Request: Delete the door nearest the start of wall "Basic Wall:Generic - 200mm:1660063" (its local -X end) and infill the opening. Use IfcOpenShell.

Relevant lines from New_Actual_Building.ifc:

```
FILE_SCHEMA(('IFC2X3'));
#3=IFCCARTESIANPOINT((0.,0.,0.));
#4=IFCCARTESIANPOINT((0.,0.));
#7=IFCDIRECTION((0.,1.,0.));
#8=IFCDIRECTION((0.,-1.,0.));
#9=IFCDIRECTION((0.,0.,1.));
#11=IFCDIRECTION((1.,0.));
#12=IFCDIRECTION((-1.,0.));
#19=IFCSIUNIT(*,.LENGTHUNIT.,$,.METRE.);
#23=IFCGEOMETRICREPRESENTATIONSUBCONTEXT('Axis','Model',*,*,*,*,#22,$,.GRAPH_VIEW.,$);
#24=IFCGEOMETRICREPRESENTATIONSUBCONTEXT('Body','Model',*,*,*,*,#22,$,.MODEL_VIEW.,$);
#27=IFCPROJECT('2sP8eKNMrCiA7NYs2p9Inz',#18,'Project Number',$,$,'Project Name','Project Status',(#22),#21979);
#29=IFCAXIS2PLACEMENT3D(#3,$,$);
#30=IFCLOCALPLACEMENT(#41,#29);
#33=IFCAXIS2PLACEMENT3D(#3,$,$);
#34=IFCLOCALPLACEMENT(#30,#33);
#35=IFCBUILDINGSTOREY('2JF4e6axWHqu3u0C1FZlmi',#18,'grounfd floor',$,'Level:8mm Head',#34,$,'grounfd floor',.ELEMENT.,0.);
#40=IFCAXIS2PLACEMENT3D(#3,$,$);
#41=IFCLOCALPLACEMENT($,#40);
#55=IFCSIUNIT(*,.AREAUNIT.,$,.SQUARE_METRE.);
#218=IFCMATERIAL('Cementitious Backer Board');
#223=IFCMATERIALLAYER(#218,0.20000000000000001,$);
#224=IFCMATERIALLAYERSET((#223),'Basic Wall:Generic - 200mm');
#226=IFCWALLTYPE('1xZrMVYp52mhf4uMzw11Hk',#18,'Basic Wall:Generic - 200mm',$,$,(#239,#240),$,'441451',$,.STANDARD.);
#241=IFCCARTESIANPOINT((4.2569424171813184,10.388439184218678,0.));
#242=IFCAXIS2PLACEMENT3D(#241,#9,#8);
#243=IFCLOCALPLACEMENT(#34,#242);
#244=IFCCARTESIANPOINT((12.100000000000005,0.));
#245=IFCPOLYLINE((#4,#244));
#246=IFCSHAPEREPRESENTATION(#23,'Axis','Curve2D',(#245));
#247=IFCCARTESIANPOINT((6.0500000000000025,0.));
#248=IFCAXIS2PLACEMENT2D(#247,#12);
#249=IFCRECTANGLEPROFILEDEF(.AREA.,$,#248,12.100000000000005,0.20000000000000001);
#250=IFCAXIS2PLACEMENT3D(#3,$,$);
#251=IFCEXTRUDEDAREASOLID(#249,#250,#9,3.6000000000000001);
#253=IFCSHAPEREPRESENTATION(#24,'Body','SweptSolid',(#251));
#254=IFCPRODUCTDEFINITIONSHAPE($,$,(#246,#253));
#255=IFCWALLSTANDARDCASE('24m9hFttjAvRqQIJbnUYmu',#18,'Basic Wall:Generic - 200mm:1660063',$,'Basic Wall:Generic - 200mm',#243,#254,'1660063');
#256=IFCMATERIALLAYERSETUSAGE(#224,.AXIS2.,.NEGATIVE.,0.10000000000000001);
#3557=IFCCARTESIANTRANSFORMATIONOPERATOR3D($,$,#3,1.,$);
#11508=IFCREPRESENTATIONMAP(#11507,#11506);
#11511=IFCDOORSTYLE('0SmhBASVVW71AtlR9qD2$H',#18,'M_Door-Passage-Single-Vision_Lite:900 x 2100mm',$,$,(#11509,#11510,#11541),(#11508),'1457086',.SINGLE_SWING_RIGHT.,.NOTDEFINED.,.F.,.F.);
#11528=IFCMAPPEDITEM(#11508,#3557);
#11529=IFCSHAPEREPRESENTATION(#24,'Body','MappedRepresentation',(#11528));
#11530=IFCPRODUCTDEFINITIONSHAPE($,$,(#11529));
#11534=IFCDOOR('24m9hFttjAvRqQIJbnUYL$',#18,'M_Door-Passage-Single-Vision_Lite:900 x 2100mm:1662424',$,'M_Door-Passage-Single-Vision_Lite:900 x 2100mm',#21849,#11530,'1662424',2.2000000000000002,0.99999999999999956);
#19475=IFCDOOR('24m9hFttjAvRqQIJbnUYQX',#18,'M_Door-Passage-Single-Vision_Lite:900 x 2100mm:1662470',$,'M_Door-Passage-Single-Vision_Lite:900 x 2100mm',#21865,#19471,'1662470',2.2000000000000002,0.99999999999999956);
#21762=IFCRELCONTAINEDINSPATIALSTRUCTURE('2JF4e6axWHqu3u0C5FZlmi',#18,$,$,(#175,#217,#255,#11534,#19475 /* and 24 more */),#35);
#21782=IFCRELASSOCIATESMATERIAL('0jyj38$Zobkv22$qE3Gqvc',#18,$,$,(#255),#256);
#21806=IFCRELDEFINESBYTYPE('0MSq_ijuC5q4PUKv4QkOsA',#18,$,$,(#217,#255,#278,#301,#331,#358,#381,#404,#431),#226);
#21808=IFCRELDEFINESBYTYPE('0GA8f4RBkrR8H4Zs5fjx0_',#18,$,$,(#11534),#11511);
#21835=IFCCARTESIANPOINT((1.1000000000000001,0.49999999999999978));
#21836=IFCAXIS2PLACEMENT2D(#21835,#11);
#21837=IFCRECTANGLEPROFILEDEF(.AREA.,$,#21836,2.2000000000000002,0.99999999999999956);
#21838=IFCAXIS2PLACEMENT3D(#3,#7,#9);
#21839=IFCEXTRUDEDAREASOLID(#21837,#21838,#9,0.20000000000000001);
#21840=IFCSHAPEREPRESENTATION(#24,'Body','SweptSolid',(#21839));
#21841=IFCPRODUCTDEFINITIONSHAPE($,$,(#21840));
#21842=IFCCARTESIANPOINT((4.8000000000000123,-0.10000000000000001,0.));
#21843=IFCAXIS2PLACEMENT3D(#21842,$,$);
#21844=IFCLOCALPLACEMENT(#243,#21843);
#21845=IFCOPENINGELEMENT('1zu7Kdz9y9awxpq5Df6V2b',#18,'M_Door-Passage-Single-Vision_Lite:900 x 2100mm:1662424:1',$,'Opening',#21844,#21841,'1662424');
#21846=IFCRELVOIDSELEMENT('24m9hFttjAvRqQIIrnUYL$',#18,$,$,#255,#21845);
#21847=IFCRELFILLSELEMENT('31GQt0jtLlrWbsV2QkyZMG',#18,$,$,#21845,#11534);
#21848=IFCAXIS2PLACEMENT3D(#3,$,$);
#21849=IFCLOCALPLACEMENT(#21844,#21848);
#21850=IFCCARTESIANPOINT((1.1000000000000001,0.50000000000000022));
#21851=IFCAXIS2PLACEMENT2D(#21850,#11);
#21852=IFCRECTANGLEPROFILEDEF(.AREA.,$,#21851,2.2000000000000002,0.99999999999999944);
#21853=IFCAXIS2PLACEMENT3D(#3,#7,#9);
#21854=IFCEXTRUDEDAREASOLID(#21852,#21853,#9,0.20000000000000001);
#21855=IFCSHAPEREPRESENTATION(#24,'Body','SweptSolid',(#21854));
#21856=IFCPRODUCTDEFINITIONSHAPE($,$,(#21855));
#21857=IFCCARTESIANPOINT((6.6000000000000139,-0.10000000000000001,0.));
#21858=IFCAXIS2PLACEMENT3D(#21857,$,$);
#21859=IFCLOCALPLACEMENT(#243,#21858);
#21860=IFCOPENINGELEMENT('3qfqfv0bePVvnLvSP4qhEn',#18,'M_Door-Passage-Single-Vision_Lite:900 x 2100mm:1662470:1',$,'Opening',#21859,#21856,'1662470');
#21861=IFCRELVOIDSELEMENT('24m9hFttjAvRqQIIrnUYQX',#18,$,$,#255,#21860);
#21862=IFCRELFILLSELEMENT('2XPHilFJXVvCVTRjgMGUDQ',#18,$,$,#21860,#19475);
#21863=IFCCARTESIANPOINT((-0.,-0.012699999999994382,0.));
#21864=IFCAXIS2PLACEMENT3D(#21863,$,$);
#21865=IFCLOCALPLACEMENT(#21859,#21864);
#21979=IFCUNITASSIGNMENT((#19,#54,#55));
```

```python
import ifcopenshell
import ifcopenshell.api.feature
import ifcopenshell.api.root
import ifcopenshell.geom
import ifcopenshell.util.shape

model = ifcopenshell.open("New_Actual_Building.ifc")
settings = ifcopenshell.geom.settings()


def volume(element):
    """Net volume in cubic metres, openings subtracted."""
    shape = ifcopenshell.geom.create_shape(settings, element)
    return ifcopenshell.util.shape.get_volume(shape.geometry)


door = model.by_guid("24m9hFttjAvRqQIJbnUYL$")
opening = door.FillsVoids[0].RelatingOpeningElement
wall = opening.VoidsElements[0].RelatingBuildingElement
before = volume(wall)

ifcopenshell.api.root.remove_product(model, product=door)
ifcopenshell.api.feature.remove_feature(model, feature=opening)

after = volume(wall)

print(f"wall volume {before:.3f} -> {after:.3f} m3")

model.write("New_Actual_Building_updated.ifc")
```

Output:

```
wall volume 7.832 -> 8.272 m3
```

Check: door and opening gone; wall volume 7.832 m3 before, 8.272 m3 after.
